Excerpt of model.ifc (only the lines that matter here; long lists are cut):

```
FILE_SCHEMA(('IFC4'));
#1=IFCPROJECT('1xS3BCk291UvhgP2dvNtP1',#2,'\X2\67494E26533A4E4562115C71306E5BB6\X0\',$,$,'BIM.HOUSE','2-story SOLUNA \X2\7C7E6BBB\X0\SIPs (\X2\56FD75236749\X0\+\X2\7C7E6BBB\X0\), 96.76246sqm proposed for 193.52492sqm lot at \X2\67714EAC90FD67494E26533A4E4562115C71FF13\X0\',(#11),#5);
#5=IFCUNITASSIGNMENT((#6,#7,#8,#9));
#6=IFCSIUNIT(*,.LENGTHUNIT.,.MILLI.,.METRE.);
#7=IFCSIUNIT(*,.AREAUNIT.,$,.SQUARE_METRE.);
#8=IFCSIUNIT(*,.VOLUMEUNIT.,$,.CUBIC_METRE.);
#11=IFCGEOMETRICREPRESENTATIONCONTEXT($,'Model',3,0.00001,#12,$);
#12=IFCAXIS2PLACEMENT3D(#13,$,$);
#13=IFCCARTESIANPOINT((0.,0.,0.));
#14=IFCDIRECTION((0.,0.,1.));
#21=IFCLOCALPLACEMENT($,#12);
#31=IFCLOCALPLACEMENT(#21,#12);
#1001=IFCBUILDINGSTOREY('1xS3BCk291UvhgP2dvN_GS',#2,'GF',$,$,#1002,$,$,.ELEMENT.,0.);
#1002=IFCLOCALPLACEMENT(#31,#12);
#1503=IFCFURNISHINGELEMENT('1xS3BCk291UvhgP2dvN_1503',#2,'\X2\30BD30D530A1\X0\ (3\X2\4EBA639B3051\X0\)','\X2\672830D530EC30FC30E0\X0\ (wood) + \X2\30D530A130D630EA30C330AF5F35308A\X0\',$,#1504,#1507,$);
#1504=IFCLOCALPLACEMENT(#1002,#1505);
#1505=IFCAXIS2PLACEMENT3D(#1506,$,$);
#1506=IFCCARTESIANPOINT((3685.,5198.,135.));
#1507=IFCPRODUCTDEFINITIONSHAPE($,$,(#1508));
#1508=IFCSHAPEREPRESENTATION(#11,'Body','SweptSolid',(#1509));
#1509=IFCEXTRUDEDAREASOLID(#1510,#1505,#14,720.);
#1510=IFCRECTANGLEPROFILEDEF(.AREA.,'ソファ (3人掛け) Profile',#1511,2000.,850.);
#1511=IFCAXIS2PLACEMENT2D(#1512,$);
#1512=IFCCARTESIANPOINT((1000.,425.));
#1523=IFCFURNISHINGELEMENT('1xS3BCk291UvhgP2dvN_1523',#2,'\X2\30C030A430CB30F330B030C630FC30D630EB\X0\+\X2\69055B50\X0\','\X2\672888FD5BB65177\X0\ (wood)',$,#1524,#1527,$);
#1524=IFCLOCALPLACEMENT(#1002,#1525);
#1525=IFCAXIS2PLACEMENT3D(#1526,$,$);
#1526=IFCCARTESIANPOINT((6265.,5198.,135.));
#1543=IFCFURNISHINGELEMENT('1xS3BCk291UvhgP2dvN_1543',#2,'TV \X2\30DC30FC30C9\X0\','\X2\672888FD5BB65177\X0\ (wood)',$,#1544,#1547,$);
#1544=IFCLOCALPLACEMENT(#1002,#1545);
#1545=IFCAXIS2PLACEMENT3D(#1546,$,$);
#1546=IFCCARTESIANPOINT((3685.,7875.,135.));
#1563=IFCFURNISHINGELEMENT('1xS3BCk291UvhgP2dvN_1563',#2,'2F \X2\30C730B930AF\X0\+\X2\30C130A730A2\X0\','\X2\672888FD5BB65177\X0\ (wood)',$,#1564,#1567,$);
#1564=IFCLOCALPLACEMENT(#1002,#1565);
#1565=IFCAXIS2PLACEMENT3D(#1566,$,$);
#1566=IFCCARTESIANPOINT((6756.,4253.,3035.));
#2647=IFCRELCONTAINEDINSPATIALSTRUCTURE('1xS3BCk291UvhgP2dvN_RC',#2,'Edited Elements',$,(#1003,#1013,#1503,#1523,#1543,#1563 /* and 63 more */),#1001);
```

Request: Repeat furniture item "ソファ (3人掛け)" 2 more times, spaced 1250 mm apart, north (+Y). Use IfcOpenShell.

```python
import numpy as np
import ifcopenshell
import ifcopenshell.api.geometry
import ifcopenshell.api.root
import ifcopenshell.util.element
import ifcopenshell.util.placement

model = ifcopenshell.open("model.ifc")


def reuse_history(source, copy):
    """copy_class also copies each property set's owner history, people and application; keep the originals."""
    for rel in copy.IsDefinedBy:
        if rel.is_a("IfcRelDefinesByProperties") and (history := rel.RelatingPropertyDefinition.OwnerHistory):
            rel.RelatingPropertyDefinition.OwnerHistory = source.OwnerHistory
            ifcopenshell.util.element.remove_deep2(model, history)


source = model.by_guid("1xS3BCk291UvhgP2dvN_1503")
base = ifcopenshell.util.placement.get_local_placement(source.ObjectPlacement)
step = np.array([0.0, 1.0, 0.0]) * 1250.0

for i in range(1, 3):
    copy = ifcopenshell.api.root.copy_class(model, product=source)
    copy.Representation = ifcopenshell.util.element.copy_deep(
        model, source.Representation, exclude=["IfcGeometricRepresentationContext", "IfcRepresentationMap"]
    )
    reuse_history(source, copy)
    matrix = base.copy()
    matrix[:3, 3] += i * step
    print("added at", matrix[:3, 3].round(3) + 0.0)
    ifcopenshell.api.geometry.edit_object_placement(model, product=copy, matrix=matrix, is_si=False)

model.write("model_v2.ifc")
```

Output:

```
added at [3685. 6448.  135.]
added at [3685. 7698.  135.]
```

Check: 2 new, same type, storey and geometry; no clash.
